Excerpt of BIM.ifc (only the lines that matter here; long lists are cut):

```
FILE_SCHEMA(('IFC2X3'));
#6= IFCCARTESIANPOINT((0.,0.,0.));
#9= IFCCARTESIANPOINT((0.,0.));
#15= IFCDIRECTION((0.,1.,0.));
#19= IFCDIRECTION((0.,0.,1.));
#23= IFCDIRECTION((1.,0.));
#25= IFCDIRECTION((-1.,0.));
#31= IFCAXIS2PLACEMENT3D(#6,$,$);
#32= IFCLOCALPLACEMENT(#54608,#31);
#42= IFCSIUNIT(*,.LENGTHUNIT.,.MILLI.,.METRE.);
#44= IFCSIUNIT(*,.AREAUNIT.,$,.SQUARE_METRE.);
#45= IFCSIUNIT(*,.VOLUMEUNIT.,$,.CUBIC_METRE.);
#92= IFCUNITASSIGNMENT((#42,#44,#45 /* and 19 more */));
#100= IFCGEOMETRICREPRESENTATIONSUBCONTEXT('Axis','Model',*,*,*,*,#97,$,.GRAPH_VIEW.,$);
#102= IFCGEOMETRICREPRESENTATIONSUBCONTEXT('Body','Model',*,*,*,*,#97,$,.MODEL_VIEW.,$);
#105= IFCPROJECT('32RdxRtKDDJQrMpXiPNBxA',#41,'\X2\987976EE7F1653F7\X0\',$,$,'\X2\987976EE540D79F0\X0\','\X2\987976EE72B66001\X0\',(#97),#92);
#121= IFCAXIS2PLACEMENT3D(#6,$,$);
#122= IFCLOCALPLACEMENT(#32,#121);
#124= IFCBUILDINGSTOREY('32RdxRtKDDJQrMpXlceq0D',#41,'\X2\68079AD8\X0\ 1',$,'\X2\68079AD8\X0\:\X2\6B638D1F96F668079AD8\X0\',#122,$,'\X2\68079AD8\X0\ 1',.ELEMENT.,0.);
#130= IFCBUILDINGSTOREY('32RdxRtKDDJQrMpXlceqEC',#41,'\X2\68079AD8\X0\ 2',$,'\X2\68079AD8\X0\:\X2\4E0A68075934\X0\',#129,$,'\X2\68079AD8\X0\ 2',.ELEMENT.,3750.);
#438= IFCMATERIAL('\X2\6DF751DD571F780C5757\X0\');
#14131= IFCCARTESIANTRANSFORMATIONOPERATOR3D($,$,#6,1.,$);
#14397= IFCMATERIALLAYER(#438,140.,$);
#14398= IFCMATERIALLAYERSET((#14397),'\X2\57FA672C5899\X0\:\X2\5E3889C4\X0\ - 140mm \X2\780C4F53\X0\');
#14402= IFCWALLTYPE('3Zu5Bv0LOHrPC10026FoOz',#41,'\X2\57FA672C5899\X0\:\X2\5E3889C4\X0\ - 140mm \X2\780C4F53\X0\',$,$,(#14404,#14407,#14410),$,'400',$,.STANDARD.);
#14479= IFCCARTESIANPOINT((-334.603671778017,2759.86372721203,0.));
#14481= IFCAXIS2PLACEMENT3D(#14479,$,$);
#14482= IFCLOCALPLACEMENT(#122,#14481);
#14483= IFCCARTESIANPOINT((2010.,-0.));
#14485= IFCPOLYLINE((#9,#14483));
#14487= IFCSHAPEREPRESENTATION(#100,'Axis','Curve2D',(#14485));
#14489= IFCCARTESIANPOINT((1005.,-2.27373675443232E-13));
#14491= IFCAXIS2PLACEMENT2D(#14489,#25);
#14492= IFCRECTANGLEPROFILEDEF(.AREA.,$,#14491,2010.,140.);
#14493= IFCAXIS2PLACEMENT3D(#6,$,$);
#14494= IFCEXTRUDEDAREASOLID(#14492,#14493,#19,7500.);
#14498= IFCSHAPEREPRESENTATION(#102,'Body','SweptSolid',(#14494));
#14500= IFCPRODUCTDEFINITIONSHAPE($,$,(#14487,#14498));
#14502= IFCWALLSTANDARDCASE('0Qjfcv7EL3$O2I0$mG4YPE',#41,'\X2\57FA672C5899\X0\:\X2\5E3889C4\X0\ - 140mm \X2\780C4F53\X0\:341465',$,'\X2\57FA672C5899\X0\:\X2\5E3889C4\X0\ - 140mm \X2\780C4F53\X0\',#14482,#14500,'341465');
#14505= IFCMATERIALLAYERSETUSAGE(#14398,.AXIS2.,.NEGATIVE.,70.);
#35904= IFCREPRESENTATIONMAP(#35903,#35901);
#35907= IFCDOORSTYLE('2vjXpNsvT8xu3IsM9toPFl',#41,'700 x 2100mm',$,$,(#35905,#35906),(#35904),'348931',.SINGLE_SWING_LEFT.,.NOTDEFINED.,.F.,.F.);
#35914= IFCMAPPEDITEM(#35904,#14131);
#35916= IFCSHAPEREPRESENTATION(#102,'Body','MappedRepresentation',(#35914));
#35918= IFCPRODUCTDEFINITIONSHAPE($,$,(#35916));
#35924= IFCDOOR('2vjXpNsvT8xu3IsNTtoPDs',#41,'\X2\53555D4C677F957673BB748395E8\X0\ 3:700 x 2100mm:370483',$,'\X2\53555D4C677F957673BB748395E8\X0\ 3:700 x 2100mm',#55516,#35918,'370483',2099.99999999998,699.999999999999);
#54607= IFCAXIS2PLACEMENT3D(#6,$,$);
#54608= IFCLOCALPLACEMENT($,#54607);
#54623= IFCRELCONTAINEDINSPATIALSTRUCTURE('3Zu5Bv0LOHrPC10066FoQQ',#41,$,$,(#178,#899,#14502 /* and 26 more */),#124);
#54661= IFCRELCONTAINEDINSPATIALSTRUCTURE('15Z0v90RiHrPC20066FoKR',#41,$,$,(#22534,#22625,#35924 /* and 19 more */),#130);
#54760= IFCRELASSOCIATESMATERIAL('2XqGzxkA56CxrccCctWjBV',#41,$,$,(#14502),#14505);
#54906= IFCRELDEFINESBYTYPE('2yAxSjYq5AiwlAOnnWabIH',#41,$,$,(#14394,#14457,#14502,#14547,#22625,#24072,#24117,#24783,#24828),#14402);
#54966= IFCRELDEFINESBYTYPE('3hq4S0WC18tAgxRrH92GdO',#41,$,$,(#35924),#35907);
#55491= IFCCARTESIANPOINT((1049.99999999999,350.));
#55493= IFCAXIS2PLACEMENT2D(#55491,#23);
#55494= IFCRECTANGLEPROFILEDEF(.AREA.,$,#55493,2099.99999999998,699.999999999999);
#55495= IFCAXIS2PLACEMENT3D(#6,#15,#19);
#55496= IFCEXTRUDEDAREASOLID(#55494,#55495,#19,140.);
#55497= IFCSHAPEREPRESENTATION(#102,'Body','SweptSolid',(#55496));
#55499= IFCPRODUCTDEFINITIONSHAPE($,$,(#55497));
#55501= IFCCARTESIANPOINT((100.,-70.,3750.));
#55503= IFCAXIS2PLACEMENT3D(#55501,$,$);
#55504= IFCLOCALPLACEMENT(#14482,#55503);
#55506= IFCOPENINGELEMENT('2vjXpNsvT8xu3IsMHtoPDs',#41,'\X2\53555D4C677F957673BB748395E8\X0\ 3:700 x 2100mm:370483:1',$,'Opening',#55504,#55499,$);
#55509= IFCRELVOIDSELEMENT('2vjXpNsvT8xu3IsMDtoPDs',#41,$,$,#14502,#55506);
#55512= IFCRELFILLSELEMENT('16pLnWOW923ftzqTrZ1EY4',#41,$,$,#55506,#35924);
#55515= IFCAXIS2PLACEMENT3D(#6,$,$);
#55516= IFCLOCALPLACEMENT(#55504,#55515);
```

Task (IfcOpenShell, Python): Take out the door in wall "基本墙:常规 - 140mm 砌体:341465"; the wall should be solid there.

```python
import ifcopenshell
import ifcopenshell.api.feature
import ifcopenshell.api.root
import ifcopenshell.geom
import ifcopenshell.util.shape

model = ifcopenshell.open("BIM.ifc")
settings = ifcopenshell.geom.settings()


def volume(element):
    """Net volume in cubic metres, openings subtracted."""
    shape = ifcopenshell.geom.create_shape(settings, element)
    return ifcopenshell.util.shape.get_volume(shape.geometry)


door = model.by_id(35924)
opening = door.FillsVoids[0].RelatingOpeningElement
wall = opening.VoidsElements[0].RelatingBuildingElement
before = volume(wall)

ifcopenshell.api.root.remove_product(model, product=door)
ifcopenshell.api.feature.remove_feature(model, feature=opening)

after = volume(wall)

print(f"wall volume {before:.3f} -> {after:.3f} m3")

model.write("BIM_v2.ifc")
```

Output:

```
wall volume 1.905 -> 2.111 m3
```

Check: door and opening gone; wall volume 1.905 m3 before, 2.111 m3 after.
